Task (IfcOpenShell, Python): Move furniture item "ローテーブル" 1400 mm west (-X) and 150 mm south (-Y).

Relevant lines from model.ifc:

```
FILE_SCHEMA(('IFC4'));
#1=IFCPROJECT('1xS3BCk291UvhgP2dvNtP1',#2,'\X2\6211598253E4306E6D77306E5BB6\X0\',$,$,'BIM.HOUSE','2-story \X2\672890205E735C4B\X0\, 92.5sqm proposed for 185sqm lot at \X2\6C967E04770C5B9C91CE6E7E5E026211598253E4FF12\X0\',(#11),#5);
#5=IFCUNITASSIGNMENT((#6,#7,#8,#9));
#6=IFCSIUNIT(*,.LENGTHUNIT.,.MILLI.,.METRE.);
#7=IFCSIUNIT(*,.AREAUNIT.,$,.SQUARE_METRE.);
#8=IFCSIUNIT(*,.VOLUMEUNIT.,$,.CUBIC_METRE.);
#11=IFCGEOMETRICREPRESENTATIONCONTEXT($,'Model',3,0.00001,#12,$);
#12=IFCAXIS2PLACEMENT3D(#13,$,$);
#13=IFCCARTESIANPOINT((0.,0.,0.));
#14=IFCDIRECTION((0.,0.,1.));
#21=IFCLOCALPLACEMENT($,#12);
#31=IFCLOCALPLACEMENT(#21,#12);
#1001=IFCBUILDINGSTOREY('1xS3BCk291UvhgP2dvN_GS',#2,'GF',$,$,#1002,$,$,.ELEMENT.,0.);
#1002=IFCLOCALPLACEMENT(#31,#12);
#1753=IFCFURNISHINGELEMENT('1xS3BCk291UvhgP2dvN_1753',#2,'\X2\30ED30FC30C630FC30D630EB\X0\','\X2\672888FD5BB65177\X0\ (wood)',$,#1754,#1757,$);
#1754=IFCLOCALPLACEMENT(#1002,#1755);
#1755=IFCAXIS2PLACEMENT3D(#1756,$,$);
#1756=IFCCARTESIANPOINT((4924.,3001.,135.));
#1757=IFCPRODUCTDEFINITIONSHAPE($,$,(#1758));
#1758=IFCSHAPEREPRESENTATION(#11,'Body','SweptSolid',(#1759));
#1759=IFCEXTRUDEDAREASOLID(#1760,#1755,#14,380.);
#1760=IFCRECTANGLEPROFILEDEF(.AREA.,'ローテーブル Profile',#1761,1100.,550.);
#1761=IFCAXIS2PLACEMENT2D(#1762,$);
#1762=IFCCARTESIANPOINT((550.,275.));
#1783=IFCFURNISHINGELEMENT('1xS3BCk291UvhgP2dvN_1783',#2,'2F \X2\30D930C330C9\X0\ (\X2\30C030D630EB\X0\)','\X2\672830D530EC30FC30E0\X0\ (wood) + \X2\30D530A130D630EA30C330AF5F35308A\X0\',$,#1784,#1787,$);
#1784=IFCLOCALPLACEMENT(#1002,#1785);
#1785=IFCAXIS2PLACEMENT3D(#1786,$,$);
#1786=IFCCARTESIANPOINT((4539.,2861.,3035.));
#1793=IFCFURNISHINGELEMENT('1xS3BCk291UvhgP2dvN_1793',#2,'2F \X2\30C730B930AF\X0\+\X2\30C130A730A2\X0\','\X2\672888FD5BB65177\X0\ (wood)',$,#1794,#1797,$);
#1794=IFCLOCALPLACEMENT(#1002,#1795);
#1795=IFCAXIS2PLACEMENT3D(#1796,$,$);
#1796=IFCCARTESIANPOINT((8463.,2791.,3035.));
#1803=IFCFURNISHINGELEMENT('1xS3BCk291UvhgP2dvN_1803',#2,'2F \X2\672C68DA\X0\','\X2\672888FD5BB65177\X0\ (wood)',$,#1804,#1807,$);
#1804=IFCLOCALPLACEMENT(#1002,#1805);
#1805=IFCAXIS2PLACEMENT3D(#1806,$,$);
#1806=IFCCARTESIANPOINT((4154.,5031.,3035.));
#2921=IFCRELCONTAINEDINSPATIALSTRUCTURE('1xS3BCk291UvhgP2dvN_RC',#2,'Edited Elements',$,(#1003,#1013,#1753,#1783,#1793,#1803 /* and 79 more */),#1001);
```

```python
import ifcopenshell
import ifcopenshell.api.geometry
import ifcopenshell.util.placement

model = ifcopenshell.open("model.ifc")

item = model.by_guid("1xS3BCk291UvhgP2dvN_1753")
matrix = ifcopenshell.util.placement.get_local_placement(item.ObjectPlacement)
matrix[0, 3] -= 1400.0
matrix[1, 3] -= 150.0
ifcopenshell.api.geometry.edit_object_placement(model, product=item, matrix=matrix, is_si=False)

print(ifcopenshell.util.placement.get_local_placement(item.ObjectPlacement).round(3) + 0.0)

model.write("model-out.ifc")
```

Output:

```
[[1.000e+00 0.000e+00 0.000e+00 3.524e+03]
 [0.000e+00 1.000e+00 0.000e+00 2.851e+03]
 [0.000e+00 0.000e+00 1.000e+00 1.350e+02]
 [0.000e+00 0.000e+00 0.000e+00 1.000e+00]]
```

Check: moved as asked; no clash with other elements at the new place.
